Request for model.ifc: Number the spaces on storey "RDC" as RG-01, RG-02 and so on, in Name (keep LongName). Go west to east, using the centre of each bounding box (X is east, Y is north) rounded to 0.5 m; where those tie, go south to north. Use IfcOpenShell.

First a look at what the model holds.

```python
import ifcopenshell
import ifcopenshell.util.element
import ifcopenshell.util.placement

model = ifcopenshell.open("model.ifc")
print(model.schema)
storey = next(s for s in model.by_type("IfcBuildingStorey") if s.Name == "RDC")
spaces = [e for e in ifcopenshell.util.element.get_decomposition(storey) if e.is_a("IfcSpace")]
for e in sorted(spaces, key=lambda e: e.id()):
    origin = ifcopenshell.util.placement.get_local_placement(e.ObjectPlacement)[:3, 3]
    print(e.id(), e.Name, e.LongName, origin.round(2) + 0.0, sep=" | ")
```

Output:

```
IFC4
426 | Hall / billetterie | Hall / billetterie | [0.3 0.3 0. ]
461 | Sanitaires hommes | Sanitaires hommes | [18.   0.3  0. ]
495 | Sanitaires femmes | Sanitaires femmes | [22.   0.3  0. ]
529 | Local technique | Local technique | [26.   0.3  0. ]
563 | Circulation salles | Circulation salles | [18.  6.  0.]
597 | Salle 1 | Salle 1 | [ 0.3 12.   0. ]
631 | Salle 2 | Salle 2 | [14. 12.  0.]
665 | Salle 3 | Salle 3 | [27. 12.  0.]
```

```python
import ifcopenshell
import ifcopenshell.geom
import ifcopenshell.util.element
import ifcopenshell.util.shape

model = ifcopenshell.open("model.ifc")
settings = ifcopenshell.geom.settings()
settings.set("use-world-coords", True)


def centre(element):
    shape = ifcopenshell.geom.create_shape(settings, element)
    return ifcopenshell.util.shape.get_bbox_centroid(shape.geometry)


storey = next(s for s in model.by_type("IfcBuildingStorey") if s.Name == "RDC")
spaces = [e for e in ifcopenshell.util.element.get_decomposition(storey) if e.is_a("IfcSpace")]

# Insertion points can sit at a corner or the storey origin, so sort by the geometry (in metres).
centres = {e: centre(e) for e in spaces}
spaces.sort(key=lambda e: (round(centres[e][0] / 0.5), centres[e][1]))

for i, e in enumerate(spaces, start=1):
    number = f"RG-{i:02d}"
    e.Name = number
    print(e.id(), number)

model.write("model_edited.ifc")
```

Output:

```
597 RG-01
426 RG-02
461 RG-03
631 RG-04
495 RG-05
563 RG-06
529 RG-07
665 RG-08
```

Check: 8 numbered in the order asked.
